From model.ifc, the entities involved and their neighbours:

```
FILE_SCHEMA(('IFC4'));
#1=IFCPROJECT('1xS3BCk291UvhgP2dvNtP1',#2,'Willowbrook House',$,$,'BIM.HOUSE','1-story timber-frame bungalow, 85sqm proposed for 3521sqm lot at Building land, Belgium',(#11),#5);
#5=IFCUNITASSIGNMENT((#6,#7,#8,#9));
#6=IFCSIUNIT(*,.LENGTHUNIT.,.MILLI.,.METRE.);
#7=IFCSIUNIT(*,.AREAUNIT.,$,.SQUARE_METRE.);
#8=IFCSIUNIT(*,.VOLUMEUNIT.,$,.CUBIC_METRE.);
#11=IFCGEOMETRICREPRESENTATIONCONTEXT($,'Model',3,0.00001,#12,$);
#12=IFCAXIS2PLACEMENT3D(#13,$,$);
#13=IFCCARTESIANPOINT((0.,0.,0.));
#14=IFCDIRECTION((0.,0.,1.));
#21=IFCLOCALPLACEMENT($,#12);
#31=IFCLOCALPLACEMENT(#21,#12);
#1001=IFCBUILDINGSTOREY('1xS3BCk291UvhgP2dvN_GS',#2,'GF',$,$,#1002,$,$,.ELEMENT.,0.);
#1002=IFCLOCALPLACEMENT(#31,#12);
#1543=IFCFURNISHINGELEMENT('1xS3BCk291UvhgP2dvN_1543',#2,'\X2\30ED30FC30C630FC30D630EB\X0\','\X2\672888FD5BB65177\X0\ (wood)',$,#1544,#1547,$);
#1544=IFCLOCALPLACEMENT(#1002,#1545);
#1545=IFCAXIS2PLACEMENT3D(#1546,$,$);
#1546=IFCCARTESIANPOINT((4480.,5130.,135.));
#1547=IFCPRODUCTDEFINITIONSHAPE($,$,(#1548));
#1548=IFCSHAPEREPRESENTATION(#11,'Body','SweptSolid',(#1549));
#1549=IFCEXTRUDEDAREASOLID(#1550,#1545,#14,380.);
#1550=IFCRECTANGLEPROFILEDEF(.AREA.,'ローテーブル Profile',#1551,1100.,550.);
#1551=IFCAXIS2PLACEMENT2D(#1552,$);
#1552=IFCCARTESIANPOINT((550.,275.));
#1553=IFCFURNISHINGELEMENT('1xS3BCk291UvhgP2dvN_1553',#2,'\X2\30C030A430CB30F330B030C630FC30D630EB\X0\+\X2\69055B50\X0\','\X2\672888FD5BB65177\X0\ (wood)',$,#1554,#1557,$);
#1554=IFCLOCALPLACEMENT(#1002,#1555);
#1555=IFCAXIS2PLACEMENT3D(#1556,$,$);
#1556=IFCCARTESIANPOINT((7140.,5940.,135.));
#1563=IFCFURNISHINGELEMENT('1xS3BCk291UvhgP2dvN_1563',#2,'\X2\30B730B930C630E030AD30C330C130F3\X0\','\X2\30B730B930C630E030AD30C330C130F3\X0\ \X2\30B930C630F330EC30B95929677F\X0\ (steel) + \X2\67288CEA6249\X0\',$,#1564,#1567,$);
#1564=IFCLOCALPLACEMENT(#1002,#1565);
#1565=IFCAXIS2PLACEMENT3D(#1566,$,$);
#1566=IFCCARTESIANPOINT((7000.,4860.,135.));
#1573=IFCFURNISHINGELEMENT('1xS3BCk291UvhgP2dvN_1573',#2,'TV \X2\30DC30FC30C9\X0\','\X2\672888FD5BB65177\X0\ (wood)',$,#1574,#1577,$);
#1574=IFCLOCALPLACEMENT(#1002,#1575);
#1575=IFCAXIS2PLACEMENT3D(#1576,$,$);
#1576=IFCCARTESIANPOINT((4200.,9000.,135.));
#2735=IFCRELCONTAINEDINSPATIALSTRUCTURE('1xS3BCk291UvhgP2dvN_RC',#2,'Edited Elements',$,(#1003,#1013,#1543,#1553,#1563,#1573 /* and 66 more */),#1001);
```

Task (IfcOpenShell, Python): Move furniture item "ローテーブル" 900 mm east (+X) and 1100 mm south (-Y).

```python
import ifcopenshell
import ifcopenshell.api.geometry
import ifcopenshell.util.placement

model = ifcopenshell.open("model.ifc")

item = model.by_id(1543)
matrix = ifcopenshell.util.placement.get_local_placement(item.ObjectPlacement)
matrix[0, 3] += 900.0
matrix[1, 3] -= 1100.0
ifcopenshell.api.geometry.edit_object_placement(model, product=item, matrix=matrix, is_si=False)

print(ifcopenshell.util.placement.get_local_placement(item.ObjectPlacement).round(3) + 0.0)

model.write("model_edited.ifc")
```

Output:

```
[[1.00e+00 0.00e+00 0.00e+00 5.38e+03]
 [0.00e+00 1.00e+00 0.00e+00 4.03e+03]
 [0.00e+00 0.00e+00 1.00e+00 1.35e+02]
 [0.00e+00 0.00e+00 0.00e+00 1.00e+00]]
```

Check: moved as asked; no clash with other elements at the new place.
